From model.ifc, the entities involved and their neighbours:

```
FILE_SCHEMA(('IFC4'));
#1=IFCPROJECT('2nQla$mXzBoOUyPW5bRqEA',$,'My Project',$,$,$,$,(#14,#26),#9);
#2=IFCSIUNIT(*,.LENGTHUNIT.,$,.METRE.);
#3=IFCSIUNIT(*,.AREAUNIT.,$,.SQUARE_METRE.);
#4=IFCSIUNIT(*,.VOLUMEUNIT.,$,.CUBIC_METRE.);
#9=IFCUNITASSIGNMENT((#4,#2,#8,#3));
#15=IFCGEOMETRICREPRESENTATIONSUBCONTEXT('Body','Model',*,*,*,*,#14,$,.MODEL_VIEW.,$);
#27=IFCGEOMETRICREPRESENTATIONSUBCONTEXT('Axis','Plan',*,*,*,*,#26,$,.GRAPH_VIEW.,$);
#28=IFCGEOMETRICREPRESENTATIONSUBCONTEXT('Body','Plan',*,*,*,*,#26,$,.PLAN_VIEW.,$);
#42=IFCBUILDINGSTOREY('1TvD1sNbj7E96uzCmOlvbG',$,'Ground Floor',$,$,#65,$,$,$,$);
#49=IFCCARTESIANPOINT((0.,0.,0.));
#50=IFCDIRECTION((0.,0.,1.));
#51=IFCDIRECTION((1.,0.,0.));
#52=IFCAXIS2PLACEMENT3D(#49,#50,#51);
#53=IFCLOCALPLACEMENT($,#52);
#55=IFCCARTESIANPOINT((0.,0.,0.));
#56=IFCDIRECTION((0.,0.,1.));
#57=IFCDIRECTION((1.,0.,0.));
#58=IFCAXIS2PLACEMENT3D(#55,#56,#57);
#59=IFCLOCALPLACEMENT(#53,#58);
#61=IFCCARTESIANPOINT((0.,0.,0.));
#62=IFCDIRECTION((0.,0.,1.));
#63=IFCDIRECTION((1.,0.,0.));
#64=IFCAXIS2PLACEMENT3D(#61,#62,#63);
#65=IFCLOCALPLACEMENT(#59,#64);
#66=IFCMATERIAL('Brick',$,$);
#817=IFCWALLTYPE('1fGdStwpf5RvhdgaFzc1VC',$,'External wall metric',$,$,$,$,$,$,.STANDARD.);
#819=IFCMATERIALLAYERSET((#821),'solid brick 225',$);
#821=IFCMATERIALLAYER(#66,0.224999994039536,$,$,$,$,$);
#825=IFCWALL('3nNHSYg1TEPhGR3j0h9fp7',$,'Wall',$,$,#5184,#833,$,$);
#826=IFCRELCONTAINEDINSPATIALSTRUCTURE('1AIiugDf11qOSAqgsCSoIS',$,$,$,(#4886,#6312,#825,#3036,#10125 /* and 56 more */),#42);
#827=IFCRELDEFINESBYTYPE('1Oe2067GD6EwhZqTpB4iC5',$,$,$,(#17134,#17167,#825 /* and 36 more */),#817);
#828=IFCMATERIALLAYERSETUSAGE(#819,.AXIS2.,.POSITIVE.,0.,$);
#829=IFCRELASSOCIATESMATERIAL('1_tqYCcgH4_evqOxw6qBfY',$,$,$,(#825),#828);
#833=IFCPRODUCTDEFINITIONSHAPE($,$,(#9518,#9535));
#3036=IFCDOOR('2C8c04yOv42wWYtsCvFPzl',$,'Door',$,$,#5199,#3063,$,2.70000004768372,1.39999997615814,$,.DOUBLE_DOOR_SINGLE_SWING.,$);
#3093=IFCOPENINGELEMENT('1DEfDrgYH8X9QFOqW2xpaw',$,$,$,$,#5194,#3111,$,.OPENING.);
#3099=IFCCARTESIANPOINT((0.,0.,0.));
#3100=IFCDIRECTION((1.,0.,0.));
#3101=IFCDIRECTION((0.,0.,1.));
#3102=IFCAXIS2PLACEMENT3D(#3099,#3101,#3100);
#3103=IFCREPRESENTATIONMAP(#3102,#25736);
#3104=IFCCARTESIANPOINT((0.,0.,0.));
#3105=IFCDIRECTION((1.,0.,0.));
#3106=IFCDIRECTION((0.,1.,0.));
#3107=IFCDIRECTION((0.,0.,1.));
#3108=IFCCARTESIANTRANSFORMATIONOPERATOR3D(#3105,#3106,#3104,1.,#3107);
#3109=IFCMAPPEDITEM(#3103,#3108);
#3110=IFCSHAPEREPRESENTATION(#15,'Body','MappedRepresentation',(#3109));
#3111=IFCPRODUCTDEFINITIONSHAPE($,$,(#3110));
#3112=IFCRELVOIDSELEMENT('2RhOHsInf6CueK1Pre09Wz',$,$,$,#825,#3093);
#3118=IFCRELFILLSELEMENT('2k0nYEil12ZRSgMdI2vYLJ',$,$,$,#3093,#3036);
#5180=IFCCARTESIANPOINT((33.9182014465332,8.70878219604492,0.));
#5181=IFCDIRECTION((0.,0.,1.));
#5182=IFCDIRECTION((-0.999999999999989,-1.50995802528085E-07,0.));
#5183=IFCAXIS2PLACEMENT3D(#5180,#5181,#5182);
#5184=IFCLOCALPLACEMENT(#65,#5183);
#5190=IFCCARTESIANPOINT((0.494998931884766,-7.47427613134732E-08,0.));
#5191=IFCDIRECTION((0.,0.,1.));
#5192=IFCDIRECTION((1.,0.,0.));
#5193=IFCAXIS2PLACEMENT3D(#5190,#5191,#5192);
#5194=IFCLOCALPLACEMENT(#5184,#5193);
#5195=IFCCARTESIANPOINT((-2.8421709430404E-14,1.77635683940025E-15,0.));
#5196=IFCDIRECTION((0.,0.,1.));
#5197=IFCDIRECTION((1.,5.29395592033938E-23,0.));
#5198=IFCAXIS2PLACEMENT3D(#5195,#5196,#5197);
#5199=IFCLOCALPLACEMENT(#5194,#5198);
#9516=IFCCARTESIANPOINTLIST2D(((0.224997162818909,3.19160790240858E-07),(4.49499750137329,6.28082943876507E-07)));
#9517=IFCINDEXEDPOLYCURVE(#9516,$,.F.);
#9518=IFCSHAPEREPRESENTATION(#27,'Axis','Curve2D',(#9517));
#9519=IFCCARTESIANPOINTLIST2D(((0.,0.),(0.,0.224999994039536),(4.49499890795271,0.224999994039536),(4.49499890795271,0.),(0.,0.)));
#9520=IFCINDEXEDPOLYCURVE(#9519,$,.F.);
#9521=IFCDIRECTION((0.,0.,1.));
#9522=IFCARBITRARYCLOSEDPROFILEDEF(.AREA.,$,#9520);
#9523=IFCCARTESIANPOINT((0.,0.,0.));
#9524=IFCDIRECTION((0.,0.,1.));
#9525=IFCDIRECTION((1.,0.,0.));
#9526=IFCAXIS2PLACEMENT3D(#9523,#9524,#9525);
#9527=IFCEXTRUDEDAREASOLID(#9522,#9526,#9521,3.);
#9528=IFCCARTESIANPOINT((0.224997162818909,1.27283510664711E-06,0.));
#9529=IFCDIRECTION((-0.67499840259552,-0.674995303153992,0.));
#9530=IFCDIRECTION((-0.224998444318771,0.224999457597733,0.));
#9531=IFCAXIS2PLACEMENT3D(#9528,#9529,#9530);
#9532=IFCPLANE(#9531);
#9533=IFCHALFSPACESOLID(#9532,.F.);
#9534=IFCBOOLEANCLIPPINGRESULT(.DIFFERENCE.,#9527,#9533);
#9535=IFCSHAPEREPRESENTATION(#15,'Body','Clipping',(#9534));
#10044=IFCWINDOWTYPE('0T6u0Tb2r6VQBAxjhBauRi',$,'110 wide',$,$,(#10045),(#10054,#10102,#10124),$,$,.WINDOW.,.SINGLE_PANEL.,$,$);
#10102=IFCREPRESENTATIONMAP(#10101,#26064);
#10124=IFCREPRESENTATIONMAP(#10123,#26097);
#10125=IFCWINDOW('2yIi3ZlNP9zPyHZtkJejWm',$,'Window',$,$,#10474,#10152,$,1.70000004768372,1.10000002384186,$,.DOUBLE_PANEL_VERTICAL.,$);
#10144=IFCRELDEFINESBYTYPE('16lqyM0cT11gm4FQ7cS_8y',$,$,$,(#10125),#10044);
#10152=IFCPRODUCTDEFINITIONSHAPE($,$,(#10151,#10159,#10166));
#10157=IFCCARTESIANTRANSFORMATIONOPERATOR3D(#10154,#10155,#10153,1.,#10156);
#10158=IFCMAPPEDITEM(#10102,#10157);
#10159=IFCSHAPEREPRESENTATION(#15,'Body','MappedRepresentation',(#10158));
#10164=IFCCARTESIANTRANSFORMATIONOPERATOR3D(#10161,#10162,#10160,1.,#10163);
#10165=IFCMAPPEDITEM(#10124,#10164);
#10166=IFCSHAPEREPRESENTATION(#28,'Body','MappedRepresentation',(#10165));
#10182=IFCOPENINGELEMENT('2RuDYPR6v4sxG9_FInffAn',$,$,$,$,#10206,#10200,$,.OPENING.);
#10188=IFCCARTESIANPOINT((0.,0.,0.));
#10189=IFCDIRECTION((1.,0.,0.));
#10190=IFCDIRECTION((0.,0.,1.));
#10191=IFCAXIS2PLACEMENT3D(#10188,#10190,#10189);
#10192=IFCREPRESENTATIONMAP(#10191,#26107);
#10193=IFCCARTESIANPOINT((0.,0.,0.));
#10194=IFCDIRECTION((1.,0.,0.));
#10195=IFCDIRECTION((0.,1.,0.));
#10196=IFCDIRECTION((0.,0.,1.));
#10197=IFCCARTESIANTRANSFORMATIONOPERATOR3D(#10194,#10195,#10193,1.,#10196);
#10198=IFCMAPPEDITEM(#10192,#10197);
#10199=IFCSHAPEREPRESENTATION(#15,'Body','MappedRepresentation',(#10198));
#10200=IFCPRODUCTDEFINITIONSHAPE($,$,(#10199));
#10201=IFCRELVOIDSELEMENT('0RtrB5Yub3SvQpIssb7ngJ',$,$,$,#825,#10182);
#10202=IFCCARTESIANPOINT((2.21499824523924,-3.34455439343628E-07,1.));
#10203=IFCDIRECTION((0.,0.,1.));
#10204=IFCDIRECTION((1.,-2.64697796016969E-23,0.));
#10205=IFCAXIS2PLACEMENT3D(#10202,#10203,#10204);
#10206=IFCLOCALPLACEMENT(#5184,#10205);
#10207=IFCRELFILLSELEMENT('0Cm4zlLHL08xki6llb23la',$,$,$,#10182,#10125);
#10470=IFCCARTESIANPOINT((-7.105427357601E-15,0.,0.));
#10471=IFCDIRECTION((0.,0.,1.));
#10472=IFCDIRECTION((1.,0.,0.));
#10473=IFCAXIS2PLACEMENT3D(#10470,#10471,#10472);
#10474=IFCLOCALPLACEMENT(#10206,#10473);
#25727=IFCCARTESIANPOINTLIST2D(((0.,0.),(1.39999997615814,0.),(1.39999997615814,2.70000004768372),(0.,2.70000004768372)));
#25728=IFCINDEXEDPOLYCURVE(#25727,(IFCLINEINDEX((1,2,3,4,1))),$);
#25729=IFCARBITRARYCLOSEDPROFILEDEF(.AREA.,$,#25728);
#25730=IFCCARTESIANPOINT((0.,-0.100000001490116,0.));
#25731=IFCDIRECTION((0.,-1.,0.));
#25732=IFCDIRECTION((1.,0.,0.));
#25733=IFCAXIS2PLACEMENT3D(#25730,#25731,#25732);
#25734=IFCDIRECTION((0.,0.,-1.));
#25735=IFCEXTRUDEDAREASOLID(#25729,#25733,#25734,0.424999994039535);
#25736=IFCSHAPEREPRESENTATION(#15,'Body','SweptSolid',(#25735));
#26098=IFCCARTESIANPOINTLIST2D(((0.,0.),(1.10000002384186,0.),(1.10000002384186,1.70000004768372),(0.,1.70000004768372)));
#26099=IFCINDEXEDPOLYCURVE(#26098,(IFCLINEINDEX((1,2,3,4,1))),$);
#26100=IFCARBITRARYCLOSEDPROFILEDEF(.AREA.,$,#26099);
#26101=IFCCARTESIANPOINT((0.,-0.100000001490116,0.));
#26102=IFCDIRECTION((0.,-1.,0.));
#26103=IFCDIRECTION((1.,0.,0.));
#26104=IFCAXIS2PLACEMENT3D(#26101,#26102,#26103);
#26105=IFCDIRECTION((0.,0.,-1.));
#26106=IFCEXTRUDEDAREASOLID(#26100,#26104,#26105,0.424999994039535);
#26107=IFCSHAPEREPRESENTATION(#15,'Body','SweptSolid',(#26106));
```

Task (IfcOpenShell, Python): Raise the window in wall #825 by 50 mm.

```python
import numpy as np
import ifcopenshell
import ifcopenshell.api.geometry
import ifcopenshell.util.placement
import ifcopenshell.util.unit

model = ifcopenshell.open("model.ifc")
unit_scale = ifcopenshell.util.unit.calculate_unit_scale(model)

window = model.by_id(10125)
opening = window.FillsVoids[0].RelatingOpeningElement
dz = 0.05 / unit_scale

shift = np.array([0.0, 0.0, dz])
# The window is placed relative to its opening, so it follows when the opening moves.
matrix = ifcopenshell.util.placement.get_local_placement(opening.ObjectPlacement)
matrix[:3, 3] += shift
ifcopenshell.api.geometry.edit_object_placement(
    model, product=opening, matrix=matrix, is_si=False, should_transform_children=True
)

print(f"moved by {dz * unit_scale:+.3f} m")

model.write("model_updated.ifc")
```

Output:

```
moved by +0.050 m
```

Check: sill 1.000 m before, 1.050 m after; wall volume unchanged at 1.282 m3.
